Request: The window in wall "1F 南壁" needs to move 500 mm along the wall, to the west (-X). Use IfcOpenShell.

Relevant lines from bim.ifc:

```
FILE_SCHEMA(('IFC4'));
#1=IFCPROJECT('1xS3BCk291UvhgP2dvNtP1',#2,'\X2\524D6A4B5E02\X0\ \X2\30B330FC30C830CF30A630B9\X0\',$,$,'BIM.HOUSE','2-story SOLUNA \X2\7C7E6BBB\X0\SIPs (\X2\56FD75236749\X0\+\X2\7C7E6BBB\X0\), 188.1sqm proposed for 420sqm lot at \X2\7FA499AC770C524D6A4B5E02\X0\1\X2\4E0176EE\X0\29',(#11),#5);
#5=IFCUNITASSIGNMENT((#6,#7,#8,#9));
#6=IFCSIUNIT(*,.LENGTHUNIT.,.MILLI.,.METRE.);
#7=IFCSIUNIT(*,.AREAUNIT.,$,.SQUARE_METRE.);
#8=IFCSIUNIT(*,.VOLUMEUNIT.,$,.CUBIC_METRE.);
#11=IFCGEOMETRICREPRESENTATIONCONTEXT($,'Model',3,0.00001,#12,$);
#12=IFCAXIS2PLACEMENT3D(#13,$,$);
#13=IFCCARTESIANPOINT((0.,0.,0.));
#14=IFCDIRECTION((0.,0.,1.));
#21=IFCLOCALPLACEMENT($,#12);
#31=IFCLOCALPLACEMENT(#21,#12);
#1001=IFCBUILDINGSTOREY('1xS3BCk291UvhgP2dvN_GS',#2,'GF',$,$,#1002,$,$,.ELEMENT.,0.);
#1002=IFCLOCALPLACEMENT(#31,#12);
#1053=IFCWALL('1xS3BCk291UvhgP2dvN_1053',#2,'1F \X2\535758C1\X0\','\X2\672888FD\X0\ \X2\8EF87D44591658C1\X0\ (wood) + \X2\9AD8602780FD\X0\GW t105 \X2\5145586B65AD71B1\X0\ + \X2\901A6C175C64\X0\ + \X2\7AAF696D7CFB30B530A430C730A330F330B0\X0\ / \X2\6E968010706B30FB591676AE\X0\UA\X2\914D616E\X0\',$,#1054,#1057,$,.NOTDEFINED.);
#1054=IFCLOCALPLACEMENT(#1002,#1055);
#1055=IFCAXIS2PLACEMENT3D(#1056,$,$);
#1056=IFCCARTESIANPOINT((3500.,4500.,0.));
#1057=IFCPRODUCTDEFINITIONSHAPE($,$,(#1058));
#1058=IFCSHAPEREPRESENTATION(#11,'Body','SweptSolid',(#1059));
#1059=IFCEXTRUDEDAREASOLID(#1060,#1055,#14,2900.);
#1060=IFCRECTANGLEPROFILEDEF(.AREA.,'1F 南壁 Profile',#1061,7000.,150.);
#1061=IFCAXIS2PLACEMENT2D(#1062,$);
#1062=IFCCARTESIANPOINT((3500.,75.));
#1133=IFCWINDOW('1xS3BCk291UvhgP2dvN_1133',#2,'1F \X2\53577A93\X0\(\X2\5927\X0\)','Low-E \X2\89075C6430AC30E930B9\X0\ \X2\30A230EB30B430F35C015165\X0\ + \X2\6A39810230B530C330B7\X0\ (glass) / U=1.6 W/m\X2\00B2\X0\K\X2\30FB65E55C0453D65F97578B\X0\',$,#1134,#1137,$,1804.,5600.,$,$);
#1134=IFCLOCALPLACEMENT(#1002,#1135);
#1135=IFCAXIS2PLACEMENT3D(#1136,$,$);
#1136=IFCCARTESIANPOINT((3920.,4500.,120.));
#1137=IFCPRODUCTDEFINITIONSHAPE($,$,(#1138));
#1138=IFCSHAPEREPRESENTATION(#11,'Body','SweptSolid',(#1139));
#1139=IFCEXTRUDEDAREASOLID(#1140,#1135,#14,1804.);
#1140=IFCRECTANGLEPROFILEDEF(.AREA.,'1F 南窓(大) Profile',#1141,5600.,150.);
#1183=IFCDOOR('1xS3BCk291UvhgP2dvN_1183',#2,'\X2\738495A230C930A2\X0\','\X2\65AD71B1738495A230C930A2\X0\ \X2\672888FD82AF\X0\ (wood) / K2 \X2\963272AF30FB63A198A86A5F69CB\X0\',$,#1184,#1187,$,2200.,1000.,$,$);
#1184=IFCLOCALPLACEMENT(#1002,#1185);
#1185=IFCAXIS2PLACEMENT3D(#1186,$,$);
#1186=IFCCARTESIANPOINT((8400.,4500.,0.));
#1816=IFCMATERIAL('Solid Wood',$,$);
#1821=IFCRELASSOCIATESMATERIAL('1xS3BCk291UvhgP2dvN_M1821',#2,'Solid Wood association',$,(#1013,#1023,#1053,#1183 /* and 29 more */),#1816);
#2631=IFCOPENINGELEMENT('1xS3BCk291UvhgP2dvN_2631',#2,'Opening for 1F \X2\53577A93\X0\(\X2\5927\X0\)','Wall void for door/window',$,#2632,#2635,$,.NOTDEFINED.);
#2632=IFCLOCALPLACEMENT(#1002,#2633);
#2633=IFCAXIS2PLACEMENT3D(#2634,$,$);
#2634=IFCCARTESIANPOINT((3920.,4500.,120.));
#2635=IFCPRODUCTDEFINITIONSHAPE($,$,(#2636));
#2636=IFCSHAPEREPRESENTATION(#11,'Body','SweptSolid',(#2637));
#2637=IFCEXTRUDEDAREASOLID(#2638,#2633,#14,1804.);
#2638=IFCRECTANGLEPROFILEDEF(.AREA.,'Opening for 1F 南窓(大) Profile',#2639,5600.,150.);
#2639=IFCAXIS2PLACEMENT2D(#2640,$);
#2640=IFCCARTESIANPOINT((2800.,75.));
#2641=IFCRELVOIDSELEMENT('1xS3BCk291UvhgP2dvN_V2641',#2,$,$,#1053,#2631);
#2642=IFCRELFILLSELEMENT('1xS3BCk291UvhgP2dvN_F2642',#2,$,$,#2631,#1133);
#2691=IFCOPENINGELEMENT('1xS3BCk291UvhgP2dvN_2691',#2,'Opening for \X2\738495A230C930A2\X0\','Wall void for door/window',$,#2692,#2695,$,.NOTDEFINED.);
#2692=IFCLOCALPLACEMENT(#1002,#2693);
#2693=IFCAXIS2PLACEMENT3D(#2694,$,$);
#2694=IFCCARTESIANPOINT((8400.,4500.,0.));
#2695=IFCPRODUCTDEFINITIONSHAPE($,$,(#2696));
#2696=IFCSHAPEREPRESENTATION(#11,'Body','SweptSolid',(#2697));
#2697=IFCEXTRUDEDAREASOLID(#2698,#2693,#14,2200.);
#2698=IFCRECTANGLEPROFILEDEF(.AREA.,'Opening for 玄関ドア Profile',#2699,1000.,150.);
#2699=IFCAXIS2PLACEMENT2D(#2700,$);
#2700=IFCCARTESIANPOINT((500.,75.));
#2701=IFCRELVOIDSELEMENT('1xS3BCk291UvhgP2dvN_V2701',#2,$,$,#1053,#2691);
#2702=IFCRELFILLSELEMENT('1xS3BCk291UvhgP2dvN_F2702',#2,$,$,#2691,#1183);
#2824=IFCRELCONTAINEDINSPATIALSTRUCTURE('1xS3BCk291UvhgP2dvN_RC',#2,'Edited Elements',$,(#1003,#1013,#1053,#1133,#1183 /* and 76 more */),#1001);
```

```python
import ifcopenshell
import ifcopenshell.api.geometry
import ifcopenshell.util.placement

model = ifcopenshell.open("bim.ifc")

window = model.by_guid("1xS3BCk291UvhgP2dvN_1133")
opening = window.FillsVoids[0].RelatingOpeningElement
wall = opening.VoidsElements[0].RelatingBuildingElement

wall_matrix = ifcopenshell.util.placement.get_local_placement(wall.ObjectPlacement)
shift = wall_matrix[:3, 0] * -500.0
before = ifcopenshell.util.placement.get_local_placement(window.ObjectPlacement)[:3, 3].copy()

# The window is not placed relative to its opening, so move both.
for product in (opening, window):
    matrix = ifcopenshell.util.placement.get_local_placement(product.ObjectPlacement)
    matrix[:3, 3] += shift
    ifcopenshell.api.geometry.edit_object_placement(model, product=product, matrix=matrix, is_si=False)

after = ifcopenshell.util.placement.get_local_placement(window.ObjectPlacement)[:3, 3]
print("window moved by", (after - before).round(3) + 0.0)

model.write("bim_updated.ifc")
```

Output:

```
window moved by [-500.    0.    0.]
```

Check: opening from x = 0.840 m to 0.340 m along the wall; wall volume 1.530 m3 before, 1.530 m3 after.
